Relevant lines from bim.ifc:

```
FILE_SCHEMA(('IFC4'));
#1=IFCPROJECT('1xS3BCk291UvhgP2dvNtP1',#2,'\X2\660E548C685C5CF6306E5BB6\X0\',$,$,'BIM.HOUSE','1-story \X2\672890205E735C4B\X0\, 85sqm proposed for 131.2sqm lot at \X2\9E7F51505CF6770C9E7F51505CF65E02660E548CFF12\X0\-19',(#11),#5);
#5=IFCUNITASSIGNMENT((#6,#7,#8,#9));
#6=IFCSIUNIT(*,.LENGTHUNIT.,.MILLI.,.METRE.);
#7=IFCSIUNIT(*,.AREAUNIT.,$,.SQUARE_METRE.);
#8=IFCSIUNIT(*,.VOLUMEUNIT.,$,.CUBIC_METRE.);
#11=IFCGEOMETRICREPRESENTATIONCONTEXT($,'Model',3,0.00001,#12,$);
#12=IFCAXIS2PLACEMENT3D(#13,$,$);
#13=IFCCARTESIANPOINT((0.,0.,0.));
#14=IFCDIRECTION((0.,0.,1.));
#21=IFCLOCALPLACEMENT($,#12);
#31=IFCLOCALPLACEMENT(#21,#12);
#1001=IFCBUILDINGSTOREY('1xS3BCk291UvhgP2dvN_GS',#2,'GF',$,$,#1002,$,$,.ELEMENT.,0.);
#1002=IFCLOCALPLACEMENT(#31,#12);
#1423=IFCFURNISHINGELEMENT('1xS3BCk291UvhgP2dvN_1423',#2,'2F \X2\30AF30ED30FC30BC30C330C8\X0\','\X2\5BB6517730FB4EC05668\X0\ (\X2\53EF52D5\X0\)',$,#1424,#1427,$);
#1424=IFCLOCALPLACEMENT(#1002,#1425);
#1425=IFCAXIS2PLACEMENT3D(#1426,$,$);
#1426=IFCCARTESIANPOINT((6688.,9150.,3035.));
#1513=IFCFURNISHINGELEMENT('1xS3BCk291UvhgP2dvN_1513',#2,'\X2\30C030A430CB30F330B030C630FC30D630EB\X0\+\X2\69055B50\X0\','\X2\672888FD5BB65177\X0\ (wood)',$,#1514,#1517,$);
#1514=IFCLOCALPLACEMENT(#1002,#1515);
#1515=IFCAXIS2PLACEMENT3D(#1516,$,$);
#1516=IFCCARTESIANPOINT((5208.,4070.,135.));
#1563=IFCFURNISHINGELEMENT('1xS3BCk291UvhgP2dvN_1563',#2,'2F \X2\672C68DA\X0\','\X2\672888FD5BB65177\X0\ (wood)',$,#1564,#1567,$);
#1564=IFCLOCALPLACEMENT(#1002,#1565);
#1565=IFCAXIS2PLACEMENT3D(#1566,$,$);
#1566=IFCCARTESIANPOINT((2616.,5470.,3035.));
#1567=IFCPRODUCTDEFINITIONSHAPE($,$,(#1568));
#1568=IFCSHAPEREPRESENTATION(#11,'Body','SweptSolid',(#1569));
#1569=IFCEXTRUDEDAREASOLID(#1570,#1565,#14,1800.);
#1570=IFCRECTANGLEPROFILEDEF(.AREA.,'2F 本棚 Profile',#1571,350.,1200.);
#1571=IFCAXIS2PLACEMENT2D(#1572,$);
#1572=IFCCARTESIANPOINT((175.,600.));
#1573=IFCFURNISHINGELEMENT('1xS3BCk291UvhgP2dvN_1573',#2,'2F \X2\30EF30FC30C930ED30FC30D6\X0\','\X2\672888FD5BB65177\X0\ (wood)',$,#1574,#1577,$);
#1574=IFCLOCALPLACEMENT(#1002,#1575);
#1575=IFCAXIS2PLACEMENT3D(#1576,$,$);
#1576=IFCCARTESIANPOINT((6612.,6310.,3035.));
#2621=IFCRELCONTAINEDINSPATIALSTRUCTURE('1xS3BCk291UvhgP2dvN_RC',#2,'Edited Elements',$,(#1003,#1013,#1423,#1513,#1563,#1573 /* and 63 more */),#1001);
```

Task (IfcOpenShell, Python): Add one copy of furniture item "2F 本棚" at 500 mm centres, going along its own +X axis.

```python
import ifcopenshell
import ifcopenshell.api.geometry
import ifcopenshell.api.root
import ifcopenshell.util.element
import ifcopenshell.util.placement
import ifcopenshell.util.unit

model = ifcopenshell.open("bim.ifc")
unit_scale = ifcopenshell.util.unit.calculate_unit_scale(model)


def reuse_history(source, copy):
    """copy_class also copies each property set's owner history, people and application; keep the originals."""
    for rel in copy.IsDefinedBy:
        if rel.is_a("IfcRelDefinesByProperties") and (history := rel.RelatingPropertyDefinition.OwnerHistory):
            rel.RelatingPropertyDefinition.OwnerHistory = source.OwnerHistory
            ifcopenshell.util.element.remove_deep2(model, history)


source = model.by_id(1563)
base = ifcopenshell.util.placement.get_local_placement(source.ObjectPlacement)
step = base[:3, 0] * 0.5 / unit_scale

for i in range(1, 2):
    copy = ifcopenshell.api.root.copy_class(model, product=source)
    copy.Representation = ifcopenshell.util.element.copy_deep(
        model, source.Representation, exclude=["IfcGeometricRepresentationContext", "IfcRepresentationMap"]
    )
    reuse_history(source, copy)
    matrix = base.copy()
    matrix[:3, 3] += i * step
    print("added at", matrix[:3, 3].round(3) + 0.0)
    ifcopenshell.api.geometry.edit_object_placement(model, product=copy, matrix=matrix, is_si=False)

model.write("bim-out.ifc")
```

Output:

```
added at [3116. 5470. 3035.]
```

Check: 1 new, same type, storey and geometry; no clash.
